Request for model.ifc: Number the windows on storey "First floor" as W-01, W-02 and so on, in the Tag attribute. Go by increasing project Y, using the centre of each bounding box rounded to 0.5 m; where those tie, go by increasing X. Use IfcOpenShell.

First a look at what the model holds.

```python
import ifcopenshell
import ifcopenshell.util.element
import ifcopenshell.util.placement

model = ifcopenshell.open("model.ifc")
print(model.schema)
storey = next(s for s in model.by_type("IfcBuildingStorey") if s.Name == "First floor")
windows = [e for e in ifcopenshell.util.element.get_decomposition(storey) if e.is_a("IfcWindow")]
for e in sorted(windows, key=lambda e: e.id()):
    origin = ifcopenshell.util.placement.get_local_placement(e.ObjectPlacement)[:3, 3]
    print(e.id(), e.Tag, e.Name, origin.round(2) + 0.0, sep=" | ")
```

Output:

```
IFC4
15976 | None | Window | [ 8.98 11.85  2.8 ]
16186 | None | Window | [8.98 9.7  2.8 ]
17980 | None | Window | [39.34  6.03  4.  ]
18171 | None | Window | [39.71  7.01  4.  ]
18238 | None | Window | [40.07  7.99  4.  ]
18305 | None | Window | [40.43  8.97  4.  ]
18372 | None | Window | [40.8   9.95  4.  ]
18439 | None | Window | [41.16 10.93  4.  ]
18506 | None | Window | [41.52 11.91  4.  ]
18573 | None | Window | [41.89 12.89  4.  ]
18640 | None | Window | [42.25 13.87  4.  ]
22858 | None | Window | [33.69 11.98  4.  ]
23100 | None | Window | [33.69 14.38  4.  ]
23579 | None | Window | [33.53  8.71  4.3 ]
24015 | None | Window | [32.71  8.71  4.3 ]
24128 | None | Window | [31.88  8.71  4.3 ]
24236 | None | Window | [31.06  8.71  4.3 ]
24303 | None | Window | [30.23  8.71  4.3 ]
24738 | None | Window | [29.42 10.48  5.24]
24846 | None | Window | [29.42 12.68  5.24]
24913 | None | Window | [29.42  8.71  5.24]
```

```python
import ifcopenshell
import ifcopenshell.geom
import ifcopenshell.util.element
import ifcopenshell.util.shape

model = ifcopenshell.open("model.ifc")
settings = ifcopenshell.geom.settings()
settings.set("use-world-coords", True)


def centre(element):
    shape = ifcopenshell.geom.create_shape(settings, element)
    return ifcopenshell.util.shape.get_bbox_centroid(shape.geometry)


storey = next(s for s in model.by_type("IfcBuildingStorey") if s.Name == "First floor")
windows = [e for e in ifcopenshell.util.element.get_decomposition(storey) if e.is_a("IfcWindow")]

# Insertion points can sit at a corner or the storey origin, so sort by the geometry (in metres).
centres = {e: centre(e) for e in windows}
windows.sort(key=lambda e: (round(centres[e][1] / 0.5), centres[e][0]))

for i, e in enumerate(windows, start=1):
    number = f"W-{i:02d}"
    e.Tag = number
    print(e.id(), number)

model.write("model-out.ifc")
```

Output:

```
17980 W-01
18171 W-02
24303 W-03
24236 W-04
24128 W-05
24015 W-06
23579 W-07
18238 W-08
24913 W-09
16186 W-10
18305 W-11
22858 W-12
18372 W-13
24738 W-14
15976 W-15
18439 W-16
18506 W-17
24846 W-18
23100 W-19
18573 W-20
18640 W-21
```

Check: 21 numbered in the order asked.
